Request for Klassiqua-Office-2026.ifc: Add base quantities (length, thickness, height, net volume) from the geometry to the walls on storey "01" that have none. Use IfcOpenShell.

First a look at what the model holds.

```python
import ifcopenshell
import ifcopenshell.util.element
import ifcopenshell.util.unit

model = ifcopenshell.open("Klassiqua-Office-2026.ifc")
print(model.schema)
for unit_type in ("LENGTHUNIT", "AREAUNIT", "VOLUMEUNIT"):
    print(unit_type, ifcopenshell.util.unit.calculate_unit_scale(model, unit_type))
storey = next(s for s in model.by_type("IfcBuildingStorey") if s.Name == "01")
walls = [e for e in ifcopenshell.util.element.get_decomposition(storey) if e.is_a("IfcWall")]
for e in sorted(walls, key=lambda e: e.id()):
    print(e.id(), e.is_a(), e.Name, list(ifcopenshell.util.element.get_psets(e, qtos_only=True)), sep=" | ")
```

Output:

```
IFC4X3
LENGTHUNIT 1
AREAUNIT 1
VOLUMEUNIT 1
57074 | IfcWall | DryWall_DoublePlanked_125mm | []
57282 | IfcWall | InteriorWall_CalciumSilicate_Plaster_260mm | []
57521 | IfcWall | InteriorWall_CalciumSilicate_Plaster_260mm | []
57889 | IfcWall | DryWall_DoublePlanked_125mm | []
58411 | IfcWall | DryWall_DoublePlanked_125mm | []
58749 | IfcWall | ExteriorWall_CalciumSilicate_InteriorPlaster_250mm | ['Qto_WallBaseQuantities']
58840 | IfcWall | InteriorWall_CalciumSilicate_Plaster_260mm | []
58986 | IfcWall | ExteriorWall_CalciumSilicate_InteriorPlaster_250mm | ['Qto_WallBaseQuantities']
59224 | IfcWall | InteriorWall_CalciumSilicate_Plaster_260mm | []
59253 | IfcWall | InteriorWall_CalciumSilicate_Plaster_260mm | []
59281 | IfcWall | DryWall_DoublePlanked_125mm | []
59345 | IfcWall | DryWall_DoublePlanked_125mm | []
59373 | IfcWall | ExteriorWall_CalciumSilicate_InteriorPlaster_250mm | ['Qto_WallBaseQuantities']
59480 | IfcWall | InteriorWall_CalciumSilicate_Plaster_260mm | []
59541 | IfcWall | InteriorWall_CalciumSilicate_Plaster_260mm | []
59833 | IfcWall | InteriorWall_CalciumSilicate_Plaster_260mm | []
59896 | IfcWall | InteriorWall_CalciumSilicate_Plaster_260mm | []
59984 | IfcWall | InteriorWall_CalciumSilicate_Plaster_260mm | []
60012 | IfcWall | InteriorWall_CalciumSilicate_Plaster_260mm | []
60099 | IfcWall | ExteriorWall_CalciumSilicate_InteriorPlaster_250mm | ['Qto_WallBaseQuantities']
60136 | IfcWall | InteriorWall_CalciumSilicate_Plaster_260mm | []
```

```python
import ifcopenshell
import ifcopenshell.api.pset
import ifcopenshell.geom
import ifcopenshell.util.element
import ifcopenshell.util.shape
import ifcopenshell.util.unit

model = ifcopenshell.open("Klassiqua-Office-2026.ifc")
unit_scale = ifcopenshell.util.unit.calculate_unit_scale(model)
volume_scale = ifcopenshell.util.unit.calculate_unit_scale(model, "VOLUMEUNIT")
settings = ifcopenshell.geom.settings()

storey = next(s for s in model.by_type("IfcBuildingStorey") if s.Name == "01")
walls = [e for e in ifcopenshell.util.element.get_decomposition(storey) if e.is_a("IfcWall")]

for e in sorted(walls, key=lambda e: e.id()):
    if ifcopenshell.util.element.get_psets(e, qtos_only=True, should_inherit=False):
        continue
    # Geometry comes back in metres, in the element's own axes.
    shape = ifcopenshell.geom.create_shape(settings, e)
    values = {
        "Length": ifcopenshell.util.shape.get_x(shape.geometry) / unit_scale,
        "Width": ifcopenshell.util.shape.get_y(shape.geometry) / unit_scale,
        "Height": ifcopenshell.util.shape.get_z(shape.geometry) / unit_scale,
        "NetVolume": ifcopenshell.util.shape.get_volume(shape.geometry) / volume_scale,
    }
    qto = ifcopenshell.api.pset.add_qto(model, product=e, name="Qto_WallBaseQuantities")
    ifcopenshell.api.pset.edit_qto(model, qto=qto, properties=values)
    print(e.id(), {k: round(v, 3) for k, v in values.items()})

model.write("Klassiqua-Office-2026_rev.ifc")
```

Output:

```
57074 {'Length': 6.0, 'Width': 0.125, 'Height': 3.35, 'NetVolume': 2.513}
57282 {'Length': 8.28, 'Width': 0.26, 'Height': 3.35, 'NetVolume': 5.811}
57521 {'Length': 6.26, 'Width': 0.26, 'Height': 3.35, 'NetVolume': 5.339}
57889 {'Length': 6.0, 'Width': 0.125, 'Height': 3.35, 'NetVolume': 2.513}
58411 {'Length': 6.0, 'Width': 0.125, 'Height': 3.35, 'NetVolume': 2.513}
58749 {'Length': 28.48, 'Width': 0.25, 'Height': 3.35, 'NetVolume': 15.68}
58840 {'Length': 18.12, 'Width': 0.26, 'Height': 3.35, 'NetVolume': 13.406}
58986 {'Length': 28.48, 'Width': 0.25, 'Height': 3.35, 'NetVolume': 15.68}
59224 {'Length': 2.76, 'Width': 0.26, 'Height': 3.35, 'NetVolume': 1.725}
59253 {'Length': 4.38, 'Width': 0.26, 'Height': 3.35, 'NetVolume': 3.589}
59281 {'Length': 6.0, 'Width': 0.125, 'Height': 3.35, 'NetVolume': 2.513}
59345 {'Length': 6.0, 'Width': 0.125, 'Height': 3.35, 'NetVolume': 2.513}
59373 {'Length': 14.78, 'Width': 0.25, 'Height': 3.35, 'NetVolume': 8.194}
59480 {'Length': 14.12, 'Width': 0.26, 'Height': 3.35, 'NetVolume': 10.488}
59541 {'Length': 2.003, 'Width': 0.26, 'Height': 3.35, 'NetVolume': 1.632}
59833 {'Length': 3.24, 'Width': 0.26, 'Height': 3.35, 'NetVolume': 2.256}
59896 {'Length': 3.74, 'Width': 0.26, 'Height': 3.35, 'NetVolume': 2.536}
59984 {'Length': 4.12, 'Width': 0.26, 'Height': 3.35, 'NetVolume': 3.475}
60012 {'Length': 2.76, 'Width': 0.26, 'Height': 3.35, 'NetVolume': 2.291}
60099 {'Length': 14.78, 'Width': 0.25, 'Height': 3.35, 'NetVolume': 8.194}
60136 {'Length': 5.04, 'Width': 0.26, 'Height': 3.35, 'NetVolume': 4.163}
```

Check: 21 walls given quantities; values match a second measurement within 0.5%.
